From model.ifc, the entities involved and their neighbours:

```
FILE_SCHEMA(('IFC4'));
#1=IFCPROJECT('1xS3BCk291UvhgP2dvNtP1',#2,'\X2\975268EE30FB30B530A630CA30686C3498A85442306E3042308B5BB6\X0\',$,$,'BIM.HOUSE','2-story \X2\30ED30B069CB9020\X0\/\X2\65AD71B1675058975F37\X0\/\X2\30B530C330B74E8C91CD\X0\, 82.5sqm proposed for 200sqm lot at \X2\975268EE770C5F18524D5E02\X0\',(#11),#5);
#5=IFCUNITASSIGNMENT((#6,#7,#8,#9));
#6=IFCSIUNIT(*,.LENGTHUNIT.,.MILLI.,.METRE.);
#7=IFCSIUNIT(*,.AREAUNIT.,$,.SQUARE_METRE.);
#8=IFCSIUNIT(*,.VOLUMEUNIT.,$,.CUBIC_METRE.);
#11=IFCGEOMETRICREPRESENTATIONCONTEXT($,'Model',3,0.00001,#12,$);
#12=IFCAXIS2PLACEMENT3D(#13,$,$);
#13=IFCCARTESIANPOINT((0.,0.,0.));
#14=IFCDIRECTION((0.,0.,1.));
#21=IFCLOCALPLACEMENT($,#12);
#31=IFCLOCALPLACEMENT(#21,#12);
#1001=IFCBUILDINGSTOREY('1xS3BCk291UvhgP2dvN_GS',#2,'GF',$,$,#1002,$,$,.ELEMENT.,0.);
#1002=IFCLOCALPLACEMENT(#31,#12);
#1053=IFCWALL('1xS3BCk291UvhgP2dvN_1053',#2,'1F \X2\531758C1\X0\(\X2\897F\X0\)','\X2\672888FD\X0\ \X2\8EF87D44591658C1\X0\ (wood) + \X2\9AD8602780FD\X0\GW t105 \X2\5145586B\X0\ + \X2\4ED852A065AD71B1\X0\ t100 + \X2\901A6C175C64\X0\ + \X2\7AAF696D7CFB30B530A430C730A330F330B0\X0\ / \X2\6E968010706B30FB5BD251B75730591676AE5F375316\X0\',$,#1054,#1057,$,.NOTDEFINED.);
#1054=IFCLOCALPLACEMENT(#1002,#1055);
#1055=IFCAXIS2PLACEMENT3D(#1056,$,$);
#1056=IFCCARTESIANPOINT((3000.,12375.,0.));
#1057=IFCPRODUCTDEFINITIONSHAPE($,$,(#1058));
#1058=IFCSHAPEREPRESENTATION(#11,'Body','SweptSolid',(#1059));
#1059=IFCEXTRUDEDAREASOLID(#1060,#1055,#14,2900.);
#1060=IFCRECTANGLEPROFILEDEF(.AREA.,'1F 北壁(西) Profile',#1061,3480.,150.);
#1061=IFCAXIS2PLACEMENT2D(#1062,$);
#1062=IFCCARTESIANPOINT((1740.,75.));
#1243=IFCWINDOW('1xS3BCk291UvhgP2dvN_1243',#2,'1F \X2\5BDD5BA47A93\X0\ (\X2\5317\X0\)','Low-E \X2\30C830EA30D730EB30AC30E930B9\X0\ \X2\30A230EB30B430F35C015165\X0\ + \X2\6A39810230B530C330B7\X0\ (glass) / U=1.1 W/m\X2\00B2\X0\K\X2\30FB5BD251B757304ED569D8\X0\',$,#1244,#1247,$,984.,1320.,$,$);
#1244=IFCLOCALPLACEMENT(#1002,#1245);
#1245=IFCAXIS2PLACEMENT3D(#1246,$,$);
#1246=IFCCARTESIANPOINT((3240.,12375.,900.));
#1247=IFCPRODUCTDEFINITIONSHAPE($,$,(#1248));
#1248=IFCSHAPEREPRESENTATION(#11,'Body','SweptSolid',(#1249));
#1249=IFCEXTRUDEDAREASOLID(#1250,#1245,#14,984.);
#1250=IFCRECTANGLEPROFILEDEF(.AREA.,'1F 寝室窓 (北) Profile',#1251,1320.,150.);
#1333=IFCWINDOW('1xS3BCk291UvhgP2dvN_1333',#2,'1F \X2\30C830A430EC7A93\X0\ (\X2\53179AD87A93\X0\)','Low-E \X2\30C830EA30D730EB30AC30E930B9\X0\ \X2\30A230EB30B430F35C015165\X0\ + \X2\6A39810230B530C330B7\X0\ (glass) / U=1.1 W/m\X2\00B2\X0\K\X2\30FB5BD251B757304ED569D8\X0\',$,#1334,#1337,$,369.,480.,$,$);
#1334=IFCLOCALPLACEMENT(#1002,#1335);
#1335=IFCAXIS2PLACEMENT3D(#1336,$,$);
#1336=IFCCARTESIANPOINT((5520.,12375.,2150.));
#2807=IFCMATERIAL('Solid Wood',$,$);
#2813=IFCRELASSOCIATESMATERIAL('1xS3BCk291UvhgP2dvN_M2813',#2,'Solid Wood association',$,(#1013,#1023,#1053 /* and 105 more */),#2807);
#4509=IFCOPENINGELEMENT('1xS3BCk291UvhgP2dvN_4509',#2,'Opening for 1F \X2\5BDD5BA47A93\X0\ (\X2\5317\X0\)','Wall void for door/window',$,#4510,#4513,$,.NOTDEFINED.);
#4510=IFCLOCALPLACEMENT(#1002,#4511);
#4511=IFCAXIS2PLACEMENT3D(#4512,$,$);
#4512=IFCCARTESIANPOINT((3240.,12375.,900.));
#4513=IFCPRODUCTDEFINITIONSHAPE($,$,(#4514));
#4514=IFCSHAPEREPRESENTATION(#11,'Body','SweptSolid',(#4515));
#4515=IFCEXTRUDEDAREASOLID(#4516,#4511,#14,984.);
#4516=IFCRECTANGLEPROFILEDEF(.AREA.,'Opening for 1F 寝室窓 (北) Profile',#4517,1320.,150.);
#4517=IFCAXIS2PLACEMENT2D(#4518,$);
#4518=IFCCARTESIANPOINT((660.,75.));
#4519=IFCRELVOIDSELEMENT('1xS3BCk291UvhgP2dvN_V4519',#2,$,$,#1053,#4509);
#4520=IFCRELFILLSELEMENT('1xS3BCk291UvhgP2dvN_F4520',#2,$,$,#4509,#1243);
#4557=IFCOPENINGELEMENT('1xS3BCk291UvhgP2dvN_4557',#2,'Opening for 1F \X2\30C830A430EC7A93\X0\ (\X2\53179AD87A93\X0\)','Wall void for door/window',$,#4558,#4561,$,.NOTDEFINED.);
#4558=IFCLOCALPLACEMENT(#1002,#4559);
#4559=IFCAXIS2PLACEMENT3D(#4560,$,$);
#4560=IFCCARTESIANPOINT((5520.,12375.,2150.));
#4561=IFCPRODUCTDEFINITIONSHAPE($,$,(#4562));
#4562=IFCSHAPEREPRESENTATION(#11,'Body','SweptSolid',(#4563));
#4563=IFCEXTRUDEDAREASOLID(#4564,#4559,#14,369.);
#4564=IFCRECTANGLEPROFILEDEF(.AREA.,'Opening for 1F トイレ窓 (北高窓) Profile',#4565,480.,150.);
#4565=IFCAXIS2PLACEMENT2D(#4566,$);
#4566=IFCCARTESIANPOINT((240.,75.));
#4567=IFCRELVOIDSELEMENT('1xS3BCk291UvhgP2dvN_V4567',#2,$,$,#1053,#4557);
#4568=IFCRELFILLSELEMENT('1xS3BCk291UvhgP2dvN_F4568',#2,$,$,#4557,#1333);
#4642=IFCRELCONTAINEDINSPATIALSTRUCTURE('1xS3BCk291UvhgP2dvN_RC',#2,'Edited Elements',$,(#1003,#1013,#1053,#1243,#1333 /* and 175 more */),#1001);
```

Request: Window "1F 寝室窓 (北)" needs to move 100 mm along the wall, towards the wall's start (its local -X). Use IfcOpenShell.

```python
import ifcopenshell
import ifcopenshell.api.geometry
import ifcopenshell.util.placement
import ifcopenshell.util.unit

model = ifcopenshell.open("model.ifc")
unit_scale = ifcopenshell.util.unit.calculate_unit_scale(model)

window = model.by_id(1243)
opening = window.FillsVoids[0].RelatingOpeningElement
wall = opening.VoidsElements[0].RelatingBuildingElement

wall_matrix = ifcopenshell.util.placement.get_local_placement(wall.ObjectPlacement)
shift = wall_matrix[:3, 0] * -0.1 / unit_scale
before = ifcopenshell.util.placement.get_local_placement(window.ObjectPlacement)[:3, 3].copy()

# The window is not placed relative to its opening, so move both.
for product in (opening, window):
    matrix = ifcopenshell.util.placement.get_local_placement(product.ObjectPlacement)
    matrix[:3, 3] += shift
    ifcopenshell.api.geometry.edit_object_placement(model, product=product, matrix=matrix, is_si=False)

after = ifcopenshell.util.placement.get_local_placement(window.ObjectPlacement)[:3, 3]
print("window moved by", (after - before).round(3) + 0.0)

model.write("model_rev.ifc")
```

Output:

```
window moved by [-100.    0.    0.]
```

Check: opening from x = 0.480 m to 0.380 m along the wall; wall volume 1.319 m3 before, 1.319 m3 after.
